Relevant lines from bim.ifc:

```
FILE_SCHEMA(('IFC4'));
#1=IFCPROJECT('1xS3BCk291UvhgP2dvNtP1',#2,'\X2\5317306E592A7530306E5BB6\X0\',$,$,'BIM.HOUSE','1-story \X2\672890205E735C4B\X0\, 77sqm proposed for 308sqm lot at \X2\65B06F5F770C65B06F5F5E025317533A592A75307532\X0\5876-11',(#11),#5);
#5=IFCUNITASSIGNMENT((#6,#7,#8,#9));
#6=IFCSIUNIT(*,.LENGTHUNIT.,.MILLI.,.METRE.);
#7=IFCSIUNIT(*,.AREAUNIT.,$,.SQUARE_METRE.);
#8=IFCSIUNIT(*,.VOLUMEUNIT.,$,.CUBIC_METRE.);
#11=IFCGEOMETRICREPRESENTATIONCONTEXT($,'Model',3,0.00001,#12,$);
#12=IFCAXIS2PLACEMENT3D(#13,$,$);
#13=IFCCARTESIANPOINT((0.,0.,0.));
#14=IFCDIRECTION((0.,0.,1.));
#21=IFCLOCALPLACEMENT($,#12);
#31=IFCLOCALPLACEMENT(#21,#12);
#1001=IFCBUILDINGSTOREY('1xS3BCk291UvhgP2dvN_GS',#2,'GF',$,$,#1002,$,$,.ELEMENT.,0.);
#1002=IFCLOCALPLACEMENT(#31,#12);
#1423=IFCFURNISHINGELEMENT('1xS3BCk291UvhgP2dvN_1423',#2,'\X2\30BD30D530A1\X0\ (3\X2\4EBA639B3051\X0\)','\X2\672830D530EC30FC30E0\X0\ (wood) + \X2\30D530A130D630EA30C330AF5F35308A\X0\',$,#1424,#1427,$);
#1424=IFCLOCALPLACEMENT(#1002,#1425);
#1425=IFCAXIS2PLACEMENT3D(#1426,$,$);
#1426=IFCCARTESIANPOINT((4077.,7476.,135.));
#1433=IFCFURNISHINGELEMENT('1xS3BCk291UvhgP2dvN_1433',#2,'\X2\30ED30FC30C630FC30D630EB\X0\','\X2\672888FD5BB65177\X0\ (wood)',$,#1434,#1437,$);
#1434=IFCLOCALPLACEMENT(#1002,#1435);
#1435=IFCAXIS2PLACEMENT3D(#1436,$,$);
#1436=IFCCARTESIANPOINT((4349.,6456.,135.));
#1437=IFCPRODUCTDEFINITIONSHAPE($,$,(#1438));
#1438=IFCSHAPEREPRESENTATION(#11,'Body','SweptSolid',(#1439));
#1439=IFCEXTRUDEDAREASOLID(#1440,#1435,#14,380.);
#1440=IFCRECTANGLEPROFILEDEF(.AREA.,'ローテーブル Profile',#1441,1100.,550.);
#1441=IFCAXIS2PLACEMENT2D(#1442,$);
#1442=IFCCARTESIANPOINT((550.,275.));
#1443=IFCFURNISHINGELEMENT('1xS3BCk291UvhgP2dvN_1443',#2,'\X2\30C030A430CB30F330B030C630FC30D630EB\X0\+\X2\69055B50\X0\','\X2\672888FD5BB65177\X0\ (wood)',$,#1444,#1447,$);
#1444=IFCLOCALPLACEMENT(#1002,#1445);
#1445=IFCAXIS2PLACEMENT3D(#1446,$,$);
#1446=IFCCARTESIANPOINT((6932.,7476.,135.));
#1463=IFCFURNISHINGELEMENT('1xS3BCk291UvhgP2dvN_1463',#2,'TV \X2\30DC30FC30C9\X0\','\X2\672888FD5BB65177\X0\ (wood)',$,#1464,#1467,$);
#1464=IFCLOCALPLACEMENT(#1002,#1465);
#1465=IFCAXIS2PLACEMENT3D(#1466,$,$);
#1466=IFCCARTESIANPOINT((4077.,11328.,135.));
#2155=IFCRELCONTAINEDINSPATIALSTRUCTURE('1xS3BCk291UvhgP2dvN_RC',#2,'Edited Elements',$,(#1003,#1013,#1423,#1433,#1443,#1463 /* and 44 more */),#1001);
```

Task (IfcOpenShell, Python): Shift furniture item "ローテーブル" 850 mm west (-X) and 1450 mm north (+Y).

```python
import ifcopenshell
import ifcopenshell.api.geometry
import ifcopenshell.util.placement
import ifcopenshell.util.unit

model = ifcopenshell.open("bim.ifc")
unit_scale = ifcopenshell.util.unit.calculate_unit_scale(model)

item = model.by_id(1433)
matrix = ifcopenshell.util.placement.get_local_placement(item.ObjectPlacement)
matrix[0, 3] -= 0.85 / unit_scale
matrix[1, 3] += 1.45 / unit_scale
ifcopenshell.api.geometry.edit_object_placement(model, product=item, matrix=matrix, is_si=False)

print(ifcopenshell.util.placement.get_local_placement(item.ObjectPlacement).round(3) + 0.0)

model.write("bim-out.ifc")
```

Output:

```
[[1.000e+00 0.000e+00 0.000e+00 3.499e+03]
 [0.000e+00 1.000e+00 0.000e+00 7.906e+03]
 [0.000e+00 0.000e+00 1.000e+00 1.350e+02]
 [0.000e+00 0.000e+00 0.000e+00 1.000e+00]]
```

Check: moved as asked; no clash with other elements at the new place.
